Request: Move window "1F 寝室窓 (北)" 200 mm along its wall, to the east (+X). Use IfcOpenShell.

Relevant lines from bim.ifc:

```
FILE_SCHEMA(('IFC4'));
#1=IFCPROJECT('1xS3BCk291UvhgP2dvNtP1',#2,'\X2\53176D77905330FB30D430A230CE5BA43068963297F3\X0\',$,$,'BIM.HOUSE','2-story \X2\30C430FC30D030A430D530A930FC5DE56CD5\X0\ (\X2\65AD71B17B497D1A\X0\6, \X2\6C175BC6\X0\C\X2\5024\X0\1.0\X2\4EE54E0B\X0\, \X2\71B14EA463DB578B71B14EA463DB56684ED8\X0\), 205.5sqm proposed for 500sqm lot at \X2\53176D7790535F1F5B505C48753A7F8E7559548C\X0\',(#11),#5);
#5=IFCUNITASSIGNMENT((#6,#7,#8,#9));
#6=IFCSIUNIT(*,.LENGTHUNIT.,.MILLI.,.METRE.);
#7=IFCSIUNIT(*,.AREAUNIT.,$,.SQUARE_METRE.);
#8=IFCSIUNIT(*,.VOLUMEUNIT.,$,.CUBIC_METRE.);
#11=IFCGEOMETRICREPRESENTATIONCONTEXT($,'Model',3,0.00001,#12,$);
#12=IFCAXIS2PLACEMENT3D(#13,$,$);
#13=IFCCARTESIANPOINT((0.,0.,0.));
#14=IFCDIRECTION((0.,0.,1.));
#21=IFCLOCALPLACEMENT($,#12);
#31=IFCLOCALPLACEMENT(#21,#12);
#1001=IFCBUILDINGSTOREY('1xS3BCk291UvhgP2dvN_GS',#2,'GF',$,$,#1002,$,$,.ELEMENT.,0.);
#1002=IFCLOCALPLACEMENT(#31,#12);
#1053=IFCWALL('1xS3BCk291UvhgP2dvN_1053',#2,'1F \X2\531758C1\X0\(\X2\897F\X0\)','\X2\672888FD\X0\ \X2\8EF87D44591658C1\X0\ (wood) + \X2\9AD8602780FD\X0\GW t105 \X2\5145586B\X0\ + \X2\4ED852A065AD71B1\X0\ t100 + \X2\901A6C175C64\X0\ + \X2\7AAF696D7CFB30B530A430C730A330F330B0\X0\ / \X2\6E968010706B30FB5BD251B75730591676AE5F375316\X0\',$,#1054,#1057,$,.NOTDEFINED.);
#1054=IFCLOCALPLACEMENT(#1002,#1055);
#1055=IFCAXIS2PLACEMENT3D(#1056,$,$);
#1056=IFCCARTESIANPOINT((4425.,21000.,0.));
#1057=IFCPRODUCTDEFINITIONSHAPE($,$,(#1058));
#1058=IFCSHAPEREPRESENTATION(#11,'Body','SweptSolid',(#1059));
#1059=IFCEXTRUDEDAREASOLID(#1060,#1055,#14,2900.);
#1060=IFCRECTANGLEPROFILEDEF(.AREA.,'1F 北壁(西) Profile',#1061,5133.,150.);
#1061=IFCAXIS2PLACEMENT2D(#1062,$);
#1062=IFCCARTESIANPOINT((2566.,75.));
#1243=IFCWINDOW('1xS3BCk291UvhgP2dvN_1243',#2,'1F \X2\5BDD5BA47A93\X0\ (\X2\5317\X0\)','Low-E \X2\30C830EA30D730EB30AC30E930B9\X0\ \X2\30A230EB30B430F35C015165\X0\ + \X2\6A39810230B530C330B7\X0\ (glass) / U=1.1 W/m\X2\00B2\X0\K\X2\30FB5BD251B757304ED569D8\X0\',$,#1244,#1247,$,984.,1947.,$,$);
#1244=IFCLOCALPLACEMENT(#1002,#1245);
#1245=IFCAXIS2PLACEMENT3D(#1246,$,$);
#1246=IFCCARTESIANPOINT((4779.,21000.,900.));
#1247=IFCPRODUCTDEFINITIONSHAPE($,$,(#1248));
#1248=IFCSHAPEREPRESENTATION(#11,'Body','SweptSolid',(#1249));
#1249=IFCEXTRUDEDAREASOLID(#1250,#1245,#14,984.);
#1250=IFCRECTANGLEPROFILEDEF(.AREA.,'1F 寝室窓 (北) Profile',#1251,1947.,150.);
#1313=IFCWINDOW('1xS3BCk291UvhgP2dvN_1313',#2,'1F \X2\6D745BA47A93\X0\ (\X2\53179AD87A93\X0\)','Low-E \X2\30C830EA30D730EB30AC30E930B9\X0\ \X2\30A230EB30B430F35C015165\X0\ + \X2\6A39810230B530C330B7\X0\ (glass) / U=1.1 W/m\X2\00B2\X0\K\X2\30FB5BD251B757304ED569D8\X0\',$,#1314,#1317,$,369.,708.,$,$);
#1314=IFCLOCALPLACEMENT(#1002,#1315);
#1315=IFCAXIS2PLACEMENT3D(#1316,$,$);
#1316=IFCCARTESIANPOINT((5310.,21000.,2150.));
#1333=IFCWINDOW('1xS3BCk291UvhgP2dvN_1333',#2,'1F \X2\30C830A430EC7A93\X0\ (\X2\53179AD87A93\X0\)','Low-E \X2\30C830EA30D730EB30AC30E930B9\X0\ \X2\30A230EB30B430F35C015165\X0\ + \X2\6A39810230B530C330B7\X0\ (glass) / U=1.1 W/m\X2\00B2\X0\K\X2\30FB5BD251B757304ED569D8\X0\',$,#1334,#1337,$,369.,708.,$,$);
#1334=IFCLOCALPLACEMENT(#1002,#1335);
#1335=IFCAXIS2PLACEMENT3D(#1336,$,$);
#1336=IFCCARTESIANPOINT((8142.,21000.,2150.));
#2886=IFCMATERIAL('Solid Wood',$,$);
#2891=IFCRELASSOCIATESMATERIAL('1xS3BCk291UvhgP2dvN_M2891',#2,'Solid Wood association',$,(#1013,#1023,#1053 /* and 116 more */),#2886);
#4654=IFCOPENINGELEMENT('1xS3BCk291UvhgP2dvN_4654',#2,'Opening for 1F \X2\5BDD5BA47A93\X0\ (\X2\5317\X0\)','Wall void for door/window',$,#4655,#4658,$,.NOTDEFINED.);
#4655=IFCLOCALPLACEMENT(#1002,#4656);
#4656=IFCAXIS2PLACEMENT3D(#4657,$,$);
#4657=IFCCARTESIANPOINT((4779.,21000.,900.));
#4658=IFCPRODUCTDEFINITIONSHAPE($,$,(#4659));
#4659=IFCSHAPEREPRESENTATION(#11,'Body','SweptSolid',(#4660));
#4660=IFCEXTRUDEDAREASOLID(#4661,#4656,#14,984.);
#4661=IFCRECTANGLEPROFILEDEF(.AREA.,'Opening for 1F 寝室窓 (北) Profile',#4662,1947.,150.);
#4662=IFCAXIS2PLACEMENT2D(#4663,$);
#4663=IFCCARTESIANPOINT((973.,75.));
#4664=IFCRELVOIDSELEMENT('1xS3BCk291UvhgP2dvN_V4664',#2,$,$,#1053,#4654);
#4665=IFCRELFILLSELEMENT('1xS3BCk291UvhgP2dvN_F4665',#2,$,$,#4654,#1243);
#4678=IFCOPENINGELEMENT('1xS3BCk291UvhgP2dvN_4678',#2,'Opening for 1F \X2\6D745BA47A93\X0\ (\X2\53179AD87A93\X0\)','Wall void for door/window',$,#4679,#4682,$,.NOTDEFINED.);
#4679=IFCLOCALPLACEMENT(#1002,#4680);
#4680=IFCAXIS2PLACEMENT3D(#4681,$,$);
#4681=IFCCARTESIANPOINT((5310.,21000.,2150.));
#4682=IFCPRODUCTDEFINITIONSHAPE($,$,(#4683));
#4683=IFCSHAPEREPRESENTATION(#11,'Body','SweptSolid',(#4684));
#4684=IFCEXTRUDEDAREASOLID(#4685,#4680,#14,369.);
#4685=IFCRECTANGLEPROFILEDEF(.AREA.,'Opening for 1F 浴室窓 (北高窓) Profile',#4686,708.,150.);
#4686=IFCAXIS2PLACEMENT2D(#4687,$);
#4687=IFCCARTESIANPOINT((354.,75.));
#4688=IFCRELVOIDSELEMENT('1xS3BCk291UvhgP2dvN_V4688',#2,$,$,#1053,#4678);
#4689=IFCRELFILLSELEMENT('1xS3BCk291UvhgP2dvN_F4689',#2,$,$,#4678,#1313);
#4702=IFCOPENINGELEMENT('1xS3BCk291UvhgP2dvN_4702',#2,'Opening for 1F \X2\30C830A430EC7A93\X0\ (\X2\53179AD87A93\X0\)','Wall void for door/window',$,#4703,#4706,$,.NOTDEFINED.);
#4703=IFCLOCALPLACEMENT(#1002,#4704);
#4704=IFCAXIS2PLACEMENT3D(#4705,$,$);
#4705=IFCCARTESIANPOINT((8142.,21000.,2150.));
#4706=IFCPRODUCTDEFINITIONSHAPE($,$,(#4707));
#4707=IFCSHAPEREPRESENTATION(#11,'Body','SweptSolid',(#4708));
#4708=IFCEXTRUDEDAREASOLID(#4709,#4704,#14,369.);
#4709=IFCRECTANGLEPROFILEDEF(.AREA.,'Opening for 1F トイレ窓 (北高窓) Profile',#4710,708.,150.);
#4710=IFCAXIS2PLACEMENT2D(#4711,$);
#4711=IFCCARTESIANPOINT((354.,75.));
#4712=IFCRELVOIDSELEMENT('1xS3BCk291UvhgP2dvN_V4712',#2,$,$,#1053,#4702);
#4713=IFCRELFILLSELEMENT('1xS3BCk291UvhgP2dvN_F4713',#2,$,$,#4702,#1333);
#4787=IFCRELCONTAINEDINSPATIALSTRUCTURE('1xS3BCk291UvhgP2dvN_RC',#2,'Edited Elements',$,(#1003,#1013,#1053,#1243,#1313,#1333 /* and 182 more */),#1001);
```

```python
import ifcopenshell
import ifcopenshell.api.geometry
import ifcopenshell.util.placement
import ifcopenshell.util.unit

model = ifcopenshell.open("bim.ifc")
unit_scale = ifcopenshell.util.unit.calculate_unit_scale(model)

window = model.by_guid("1xS3BCk291UvhgP2dvN_1243")
opening = window.FillsVoids[0].RelatingOpeningElement
wall = opening.VoidsElements[0].RelatingBuildingElement

wall_matrix = ifcopenshell.util.placement.get_local_placement(wall.ObjectPlacement)
shift = wall_matrix[:3, 0] * 0.2 / unit_scale
before = ifcopenshell.util.placement.get_local_placement(window.ObjectPlacement)[:3, 3].copy()

# The window is not placed relative to its opening, so move both.
for product in (opening, window):
    matrix = ifcopenshell.util.placement.get_local_placement(product.ObjectPlacement)
    matrix[:3, 3] += shift
    ifcopenshell.api.geometry.edit_object_placement(model, product=product, matrix=matrix, is_si=False)

after = ifcopenshell.util.placement.get_local_placement(window.ObjectPlacement)[:3, 3]
print("window moved by", (after - before).round(3) + 0.0)

model.write("bim_rev.ifc")
```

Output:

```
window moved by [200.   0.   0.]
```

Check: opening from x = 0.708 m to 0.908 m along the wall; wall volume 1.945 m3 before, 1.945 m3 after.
